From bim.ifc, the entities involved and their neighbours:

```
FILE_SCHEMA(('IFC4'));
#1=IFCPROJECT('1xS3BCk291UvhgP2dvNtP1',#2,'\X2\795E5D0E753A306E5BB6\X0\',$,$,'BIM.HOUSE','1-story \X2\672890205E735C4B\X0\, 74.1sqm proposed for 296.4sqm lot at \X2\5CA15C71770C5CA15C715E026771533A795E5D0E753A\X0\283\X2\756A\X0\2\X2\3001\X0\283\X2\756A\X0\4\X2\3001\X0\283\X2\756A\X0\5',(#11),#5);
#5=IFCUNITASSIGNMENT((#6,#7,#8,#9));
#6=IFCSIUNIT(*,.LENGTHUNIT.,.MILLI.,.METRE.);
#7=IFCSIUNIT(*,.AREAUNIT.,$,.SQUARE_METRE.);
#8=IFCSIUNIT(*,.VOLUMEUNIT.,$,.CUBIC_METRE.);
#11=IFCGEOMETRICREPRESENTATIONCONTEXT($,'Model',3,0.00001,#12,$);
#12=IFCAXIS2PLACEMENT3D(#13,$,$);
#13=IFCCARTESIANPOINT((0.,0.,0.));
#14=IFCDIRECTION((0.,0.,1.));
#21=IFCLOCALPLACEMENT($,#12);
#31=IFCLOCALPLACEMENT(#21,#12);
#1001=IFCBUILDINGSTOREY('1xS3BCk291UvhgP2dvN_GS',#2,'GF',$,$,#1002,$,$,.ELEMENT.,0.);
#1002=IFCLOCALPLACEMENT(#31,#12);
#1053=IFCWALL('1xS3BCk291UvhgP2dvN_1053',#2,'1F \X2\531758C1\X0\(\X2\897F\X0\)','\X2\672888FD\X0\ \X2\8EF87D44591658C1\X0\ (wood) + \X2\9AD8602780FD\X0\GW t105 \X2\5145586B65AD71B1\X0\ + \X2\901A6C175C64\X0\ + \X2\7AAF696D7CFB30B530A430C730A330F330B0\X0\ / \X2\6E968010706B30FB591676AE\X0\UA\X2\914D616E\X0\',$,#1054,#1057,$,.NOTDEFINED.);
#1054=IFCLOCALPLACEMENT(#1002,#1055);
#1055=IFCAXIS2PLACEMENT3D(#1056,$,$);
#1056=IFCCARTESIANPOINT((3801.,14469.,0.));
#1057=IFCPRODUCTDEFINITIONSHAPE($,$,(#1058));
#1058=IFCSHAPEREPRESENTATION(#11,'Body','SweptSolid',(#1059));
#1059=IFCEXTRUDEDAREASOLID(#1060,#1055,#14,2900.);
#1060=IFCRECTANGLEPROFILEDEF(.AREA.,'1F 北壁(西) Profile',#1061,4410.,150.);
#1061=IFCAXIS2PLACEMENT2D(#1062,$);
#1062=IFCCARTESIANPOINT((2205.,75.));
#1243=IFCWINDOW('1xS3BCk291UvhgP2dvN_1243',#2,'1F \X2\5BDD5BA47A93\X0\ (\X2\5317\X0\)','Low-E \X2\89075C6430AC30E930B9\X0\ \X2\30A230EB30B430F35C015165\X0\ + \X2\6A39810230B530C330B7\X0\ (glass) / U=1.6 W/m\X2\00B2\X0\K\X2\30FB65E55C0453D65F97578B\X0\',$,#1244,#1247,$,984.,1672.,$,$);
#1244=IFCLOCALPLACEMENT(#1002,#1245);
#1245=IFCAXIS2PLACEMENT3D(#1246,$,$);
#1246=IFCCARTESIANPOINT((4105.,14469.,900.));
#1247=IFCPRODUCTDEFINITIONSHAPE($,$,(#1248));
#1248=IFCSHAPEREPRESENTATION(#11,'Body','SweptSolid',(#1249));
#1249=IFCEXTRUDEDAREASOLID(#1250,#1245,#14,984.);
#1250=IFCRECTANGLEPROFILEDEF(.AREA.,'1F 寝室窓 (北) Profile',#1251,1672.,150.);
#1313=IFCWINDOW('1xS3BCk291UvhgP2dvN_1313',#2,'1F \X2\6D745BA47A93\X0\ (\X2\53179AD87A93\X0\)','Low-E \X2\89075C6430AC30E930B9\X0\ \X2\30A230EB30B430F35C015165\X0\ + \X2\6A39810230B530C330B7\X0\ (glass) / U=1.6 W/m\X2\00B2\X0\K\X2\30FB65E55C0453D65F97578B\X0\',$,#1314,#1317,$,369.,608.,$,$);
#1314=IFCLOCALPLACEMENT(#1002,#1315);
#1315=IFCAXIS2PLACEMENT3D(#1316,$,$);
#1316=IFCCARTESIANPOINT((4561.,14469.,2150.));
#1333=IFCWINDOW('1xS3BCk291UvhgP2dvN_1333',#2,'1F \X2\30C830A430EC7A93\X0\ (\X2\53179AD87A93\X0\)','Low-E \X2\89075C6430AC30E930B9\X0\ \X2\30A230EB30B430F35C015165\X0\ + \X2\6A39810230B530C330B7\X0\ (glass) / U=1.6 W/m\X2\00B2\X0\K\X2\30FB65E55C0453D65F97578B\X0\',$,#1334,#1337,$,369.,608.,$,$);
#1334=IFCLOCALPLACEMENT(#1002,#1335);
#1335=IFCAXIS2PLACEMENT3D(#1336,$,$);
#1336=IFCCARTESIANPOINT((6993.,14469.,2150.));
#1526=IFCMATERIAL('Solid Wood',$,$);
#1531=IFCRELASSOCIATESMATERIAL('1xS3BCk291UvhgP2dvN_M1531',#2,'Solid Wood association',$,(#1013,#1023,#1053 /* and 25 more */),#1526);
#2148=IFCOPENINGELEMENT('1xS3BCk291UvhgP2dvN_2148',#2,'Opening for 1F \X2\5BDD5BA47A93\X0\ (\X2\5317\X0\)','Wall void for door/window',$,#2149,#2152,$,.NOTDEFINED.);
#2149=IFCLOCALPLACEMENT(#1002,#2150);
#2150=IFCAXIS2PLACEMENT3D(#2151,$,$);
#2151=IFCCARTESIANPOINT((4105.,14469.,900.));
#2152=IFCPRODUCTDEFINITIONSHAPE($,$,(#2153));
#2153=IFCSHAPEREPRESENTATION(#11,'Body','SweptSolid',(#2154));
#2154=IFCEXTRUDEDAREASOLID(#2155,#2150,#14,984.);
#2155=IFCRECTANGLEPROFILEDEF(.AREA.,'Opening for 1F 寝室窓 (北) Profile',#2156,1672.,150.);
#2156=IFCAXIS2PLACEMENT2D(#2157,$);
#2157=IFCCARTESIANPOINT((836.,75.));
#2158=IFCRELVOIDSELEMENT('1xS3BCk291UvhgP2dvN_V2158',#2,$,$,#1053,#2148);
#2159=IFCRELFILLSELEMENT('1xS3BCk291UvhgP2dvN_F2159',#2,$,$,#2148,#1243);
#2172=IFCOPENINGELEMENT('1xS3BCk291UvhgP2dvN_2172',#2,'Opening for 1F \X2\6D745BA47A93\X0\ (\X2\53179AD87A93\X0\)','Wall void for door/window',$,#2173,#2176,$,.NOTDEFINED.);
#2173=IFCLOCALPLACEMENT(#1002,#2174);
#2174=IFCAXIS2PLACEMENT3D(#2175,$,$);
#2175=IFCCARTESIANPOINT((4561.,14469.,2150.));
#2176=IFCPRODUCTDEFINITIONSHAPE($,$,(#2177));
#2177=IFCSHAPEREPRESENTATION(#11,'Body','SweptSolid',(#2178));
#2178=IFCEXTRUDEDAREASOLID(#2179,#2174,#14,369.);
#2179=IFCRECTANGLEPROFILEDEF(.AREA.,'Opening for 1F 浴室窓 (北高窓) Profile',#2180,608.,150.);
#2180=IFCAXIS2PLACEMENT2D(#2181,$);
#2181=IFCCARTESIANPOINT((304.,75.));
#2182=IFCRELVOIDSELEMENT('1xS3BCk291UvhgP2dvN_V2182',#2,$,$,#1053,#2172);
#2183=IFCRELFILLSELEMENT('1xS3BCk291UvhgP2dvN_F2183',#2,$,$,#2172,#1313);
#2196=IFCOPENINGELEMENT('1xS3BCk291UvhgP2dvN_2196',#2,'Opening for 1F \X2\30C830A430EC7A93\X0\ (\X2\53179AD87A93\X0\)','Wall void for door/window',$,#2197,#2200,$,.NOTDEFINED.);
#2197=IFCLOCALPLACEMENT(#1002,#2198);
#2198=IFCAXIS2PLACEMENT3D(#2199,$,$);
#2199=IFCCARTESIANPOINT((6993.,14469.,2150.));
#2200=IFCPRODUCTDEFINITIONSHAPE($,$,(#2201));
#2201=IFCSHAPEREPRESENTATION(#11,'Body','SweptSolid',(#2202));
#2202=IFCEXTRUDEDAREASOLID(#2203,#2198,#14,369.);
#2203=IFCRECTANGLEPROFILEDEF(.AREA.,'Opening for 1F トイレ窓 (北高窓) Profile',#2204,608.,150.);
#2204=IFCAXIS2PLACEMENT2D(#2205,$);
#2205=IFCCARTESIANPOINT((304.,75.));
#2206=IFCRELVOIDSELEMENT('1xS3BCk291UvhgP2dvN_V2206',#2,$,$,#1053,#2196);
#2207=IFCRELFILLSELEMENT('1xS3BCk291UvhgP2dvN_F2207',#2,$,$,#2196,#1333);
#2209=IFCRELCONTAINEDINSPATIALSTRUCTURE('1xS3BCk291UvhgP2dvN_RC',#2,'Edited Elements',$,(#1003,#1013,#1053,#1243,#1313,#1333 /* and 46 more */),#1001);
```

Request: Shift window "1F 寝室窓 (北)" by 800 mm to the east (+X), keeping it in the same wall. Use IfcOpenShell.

```python
import ifcopenshell
import ifcopenshell.api.geometry
import ifcopenshell.util.placement

model = ifcopenshell.open("bim.ifc")

window = model.by_guid("1xS3BCk291UvhgP2dvN_1243")
opening = window.FillsVoids[0].RelatingOpeningElement
wall = opening.VoidsElements[0].RelatingBuildingElement

wall_matrix = ifcopenshell.util.placement.get_local_placement(wall.ObjectPlacement)
shift = wall_matrix[:3, 0] * 800.0
before = ifcopenshell.util.placement.get_local_placement(window.ObjectPlacement)[:3, 3].copy()

# The window is not placed relative to its opening, so move both.
for product in (opening, window):
    matrix = ifcopenshell.util.placement.get_local_placement(product.ObjectPlacement)
    matrix[:3, 3] += shift
    ifcopenshell.api.geometry.edit_object_placement(model, product=product, matrix=matrix, is_si=False)

after = ifcopenshell.util.placement.get_local_placement(window.ObjectPlacement)[:3, 3]
print("window moved by", (after - before).round(3) + 0.0)

model.write("bim-out.ifc")
```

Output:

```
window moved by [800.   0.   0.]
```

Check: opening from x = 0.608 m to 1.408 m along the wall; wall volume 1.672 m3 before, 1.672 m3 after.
